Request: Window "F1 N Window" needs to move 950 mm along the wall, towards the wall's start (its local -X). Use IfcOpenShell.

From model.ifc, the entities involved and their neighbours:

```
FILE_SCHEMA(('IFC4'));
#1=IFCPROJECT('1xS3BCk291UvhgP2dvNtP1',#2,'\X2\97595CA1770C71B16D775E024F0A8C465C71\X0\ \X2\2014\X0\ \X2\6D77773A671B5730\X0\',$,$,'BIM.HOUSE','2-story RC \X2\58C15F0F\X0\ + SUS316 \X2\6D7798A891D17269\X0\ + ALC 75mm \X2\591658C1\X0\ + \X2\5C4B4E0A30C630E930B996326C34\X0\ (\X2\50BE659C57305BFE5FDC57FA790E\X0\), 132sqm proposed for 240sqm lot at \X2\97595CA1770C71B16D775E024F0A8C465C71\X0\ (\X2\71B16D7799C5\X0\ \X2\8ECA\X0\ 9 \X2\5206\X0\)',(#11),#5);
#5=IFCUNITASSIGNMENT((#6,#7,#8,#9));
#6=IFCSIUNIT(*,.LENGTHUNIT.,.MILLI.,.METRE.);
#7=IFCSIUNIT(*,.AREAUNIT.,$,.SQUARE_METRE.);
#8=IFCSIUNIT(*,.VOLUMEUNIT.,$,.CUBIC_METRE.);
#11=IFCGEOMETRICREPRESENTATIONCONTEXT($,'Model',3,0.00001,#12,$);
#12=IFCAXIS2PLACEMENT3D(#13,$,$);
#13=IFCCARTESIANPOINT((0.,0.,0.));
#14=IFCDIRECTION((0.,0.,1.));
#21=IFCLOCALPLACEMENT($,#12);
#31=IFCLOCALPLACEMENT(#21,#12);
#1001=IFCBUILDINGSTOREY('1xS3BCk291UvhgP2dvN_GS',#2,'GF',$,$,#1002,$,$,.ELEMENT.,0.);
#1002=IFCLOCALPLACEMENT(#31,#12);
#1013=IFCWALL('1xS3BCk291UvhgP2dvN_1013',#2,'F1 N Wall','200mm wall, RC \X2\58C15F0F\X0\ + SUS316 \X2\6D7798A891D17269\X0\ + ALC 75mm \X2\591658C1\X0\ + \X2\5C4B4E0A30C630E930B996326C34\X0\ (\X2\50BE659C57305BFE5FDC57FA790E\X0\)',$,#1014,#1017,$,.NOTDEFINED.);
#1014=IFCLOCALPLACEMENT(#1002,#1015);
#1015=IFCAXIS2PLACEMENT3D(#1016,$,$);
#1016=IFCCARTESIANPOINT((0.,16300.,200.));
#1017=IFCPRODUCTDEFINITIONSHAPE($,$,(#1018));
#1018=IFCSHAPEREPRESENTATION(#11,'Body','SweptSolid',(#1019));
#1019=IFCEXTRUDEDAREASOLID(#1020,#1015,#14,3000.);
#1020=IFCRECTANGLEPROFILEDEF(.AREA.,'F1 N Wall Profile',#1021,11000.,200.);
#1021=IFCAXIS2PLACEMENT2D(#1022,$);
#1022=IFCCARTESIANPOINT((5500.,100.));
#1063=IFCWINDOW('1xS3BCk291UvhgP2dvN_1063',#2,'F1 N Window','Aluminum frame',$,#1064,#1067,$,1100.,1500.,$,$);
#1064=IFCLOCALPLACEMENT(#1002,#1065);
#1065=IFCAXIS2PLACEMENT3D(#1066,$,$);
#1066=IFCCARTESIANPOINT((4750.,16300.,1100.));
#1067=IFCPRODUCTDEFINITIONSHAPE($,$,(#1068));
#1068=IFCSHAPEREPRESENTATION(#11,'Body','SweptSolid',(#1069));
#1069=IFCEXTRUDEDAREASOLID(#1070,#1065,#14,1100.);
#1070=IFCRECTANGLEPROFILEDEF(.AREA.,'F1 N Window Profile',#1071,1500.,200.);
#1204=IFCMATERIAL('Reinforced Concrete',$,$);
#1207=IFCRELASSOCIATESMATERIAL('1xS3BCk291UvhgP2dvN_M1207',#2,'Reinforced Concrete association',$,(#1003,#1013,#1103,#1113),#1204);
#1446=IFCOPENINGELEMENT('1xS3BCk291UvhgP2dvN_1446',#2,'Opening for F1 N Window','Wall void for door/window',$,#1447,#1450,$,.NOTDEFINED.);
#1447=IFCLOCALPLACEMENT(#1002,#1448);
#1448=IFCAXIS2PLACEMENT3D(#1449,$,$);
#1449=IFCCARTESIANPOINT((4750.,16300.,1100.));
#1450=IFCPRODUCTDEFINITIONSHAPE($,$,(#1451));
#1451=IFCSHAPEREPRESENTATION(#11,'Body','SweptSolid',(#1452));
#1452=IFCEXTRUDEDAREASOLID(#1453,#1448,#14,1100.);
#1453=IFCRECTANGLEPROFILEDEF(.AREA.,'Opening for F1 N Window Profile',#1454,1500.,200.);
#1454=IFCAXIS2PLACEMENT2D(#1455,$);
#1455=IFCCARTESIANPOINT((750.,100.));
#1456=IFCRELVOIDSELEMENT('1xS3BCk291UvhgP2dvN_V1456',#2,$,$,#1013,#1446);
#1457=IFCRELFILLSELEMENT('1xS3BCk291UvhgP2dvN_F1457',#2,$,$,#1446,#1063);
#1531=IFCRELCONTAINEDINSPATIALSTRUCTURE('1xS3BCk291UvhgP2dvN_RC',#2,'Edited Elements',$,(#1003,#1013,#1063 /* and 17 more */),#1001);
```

```python
import ifcopenshell
import ifcopenshell.api.geometry
import ifcopenshell.util.placement
import ifcopenshell.util.unit

model = ifcopenshell.open("model.ifc")
unit_scale = ifcopenshell.util.unit.calculate_unit_scale(model)

window = model.by_id(1063)
opening = window.FillsVoids[0].RelatingOpeningElement
wall = opening.VoidsElements[0].RelatingBuildingElement

wall_matrix = ifcopenshell.util.placement.get_local_placement(wall.ObjectPlacement)
shift = wall_matrix[:3, 0] * -0.95 / unit_scale
before = ifcopenshell.util.placement.get_local_placement(window.ObjectPlacement)[:3, 3].copy()

# The window is not placed relative to its opening, so move both.
for product in (opening, window):
    matrix = ifcopenshell.util.placement.get_local_placement(product.ObjectPlacement)
    matrix[:3, 3] += shift
    ifcopenshell.api.geometry.edit_object_placement(model, product=product, matrix=matrix, is_si=False)

after = ifcopenshell.util.placement.get_local_placement(window.ObjectPlacement)[:3, 3]
print("window moved by", (after - before).round(3) + 0.0)

model.write("model_rev.ifc")
```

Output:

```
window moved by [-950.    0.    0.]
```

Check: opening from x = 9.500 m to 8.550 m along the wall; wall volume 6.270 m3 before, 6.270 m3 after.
